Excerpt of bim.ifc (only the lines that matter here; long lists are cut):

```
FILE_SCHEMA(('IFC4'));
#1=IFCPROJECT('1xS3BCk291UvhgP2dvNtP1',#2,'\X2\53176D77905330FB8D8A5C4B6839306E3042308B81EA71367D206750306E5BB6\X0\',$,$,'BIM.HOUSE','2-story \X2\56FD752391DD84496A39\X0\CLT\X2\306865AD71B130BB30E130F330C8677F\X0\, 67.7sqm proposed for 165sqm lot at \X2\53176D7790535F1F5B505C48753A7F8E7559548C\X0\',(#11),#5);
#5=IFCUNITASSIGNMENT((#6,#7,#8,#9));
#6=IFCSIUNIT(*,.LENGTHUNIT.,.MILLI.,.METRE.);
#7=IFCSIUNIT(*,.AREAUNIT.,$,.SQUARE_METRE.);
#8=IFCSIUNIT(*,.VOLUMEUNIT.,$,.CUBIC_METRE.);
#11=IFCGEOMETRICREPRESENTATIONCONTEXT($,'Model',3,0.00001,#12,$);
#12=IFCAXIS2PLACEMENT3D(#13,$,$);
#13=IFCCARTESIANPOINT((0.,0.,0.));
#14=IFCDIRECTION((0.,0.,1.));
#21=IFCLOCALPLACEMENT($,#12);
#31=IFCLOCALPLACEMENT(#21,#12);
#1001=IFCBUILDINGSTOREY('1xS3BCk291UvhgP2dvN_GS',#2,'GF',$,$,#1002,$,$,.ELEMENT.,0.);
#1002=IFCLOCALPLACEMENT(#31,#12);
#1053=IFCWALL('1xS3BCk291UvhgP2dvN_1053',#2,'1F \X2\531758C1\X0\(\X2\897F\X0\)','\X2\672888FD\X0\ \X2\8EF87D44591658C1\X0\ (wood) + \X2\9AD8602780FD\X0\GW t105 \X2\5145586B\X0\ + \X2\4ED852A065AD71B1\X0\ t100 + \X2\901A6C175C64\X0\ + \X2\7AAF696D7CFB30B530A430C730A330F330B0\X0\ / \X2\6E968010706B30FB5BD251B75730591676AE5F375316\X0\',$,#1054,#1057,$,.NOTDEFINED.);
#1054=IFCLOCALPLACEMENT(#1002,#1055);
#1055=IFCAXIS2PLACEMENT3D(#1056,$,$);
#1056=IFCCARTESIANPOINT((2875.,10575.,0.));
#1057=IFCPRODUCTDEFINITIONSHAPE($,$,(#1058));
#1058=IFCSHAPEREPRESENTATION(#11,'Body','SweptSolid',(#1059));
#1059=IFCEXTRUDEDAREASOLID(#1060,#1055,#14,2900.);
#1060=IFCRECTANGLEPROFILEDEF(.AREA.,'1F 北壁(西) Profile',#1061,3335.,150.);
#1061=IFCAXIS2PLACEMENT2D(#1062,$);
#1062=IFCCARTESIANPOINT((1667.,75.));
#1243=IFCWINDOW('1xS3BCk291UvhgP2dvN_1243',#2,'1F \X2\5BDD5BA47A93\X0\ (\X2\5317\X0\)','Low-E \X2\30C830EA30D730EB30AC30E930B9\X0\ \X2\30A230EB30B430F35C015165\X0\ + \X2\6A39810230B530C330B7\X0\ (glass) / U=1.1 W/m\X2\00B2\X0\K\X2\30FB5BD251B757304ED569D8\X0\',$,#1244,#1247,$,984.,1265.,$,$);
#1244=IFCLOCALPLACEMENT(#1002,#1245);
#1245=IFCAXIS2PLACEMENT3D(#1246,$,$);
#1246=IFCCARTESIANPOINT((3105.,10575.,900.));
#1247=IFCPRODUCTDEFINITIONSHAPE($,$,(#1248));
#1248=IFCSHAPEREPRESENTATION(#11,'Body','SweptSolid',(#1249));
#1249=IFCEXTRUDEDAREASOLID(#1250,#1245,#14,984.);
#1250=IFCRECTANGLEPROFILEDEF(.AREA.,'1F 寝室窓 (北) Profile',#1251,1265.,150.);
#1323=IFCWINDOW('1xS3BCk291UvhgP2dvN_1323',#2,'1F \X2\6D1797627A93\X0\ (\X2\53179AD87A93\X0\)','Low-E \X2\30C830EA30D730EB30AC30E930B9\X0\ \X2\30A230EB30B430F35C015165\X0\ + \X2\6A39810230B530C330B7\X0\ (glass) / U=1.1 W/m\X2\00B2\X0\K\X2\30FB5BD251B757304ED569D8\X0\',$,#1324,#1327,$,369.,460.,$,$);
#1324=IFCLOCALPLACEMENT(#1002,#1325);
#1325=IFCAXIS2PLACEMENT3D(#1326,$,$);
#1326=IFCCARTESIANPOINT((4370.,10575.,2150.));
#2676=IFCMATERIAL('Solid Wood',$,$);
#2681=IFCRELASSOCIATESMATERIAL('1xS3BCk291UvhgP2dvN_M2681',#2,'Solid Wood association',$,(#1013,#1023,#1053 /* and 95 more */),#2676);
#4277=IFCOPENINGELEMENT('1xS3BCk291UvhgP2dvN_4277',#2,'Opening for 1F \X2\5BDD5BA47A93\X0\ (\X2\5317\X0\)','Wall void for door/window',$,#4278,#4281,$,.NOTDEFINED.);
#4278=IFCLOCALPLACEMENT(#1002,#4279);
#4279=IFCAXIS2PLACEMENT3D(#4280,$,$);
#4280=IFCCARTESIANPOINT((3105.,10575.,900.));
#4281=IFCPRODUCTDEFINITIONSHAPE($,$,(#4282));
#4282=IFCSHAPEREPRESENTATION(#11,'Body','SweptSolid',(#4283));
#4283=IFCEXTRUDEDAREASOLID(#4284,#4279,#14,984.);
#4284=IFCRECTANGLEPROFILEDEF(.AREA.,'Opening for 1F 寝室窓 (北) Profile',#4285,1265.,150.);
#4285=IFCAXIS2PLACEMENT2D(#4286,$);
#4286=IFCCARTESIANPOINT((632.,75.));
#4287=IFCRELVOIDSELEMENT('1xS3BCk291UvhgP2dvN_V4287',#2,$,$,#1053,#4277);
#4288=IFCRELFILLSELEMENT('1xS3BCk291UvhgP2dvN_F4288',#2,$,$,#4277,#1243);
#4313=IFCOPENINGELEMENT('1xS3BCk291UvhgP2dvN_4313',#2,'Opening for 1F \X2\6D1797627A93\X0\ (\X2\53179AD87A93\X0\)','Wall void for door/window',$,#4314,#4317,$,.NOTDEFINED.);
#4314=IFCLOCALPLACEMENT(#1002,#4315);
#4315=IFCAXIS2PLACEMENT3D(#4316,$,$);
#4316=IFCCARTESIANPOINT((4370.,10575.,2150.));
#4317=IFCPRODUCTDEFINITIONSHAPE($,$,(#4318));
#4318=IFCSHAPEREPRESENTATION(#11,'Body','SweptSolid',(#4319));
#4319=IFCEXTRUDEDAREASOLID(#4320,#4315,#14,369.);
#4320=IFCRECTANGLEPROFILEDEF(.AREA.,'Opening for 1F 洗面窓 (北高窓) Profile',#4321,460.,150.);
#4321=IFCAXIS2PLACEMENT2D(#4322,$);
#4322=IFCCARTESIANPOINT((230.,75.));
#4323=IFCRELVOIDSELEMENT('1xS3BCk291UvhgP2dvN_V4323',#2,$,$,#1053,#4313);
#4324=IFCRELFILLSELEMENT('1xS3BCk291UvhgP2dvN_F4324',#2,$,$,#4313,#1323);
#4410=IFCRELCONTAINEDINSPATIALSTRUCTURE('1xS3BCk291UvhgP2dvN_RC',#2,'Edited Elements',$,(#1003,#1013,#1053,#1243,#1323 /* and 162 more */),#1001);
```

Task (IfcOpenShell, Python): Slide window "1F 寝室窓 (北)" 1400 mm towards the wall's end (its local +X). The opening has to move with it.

```python
import ifcopenshell
import ifcopenshell.api.geometry
import ifcopenshell.util.placement

model = ifcopenshell.open("bim.ifc")

window = model.by_guid("1xS3BCk291UvhgP2dvN_1243")
opening = window.FillsVoids[0].RelatingOpeningElement
wall = opening.VoidsElements[0].RelatingBuildingElement

wall_matrix = ifcopenshell.util.placement.get_local_placement(wall.ObjectPlacement)
shift = wall_matrix[:3, 0] * 1400.0
before = ifcopenshell.util.placement.get_local_placement(window.ObjectPlacement)[:3, 3].copy()

# The window is not placed relative to its opening, so move both.
for product in (opening, window):
    matrix = ifcopenshell.util.placement.get_local_placement(product.ObjectPlacement)
    matrix[:3, 3] += shift
    ifcopenshell.api.geometry.edit_object_placement(model, product=product, matrix=matrix, is_si=False)

after = ifcopenshell.util.placement.get_local_placement(window.ObjectPlacement)[:3, 3]
print("window moved by", (after - before).round(3) + 0.0)

model.write("bim_updated.ifc")
```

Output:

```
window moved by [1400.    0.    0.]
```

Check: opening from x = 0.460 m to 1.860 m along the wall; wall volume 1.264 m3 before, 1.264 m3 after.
